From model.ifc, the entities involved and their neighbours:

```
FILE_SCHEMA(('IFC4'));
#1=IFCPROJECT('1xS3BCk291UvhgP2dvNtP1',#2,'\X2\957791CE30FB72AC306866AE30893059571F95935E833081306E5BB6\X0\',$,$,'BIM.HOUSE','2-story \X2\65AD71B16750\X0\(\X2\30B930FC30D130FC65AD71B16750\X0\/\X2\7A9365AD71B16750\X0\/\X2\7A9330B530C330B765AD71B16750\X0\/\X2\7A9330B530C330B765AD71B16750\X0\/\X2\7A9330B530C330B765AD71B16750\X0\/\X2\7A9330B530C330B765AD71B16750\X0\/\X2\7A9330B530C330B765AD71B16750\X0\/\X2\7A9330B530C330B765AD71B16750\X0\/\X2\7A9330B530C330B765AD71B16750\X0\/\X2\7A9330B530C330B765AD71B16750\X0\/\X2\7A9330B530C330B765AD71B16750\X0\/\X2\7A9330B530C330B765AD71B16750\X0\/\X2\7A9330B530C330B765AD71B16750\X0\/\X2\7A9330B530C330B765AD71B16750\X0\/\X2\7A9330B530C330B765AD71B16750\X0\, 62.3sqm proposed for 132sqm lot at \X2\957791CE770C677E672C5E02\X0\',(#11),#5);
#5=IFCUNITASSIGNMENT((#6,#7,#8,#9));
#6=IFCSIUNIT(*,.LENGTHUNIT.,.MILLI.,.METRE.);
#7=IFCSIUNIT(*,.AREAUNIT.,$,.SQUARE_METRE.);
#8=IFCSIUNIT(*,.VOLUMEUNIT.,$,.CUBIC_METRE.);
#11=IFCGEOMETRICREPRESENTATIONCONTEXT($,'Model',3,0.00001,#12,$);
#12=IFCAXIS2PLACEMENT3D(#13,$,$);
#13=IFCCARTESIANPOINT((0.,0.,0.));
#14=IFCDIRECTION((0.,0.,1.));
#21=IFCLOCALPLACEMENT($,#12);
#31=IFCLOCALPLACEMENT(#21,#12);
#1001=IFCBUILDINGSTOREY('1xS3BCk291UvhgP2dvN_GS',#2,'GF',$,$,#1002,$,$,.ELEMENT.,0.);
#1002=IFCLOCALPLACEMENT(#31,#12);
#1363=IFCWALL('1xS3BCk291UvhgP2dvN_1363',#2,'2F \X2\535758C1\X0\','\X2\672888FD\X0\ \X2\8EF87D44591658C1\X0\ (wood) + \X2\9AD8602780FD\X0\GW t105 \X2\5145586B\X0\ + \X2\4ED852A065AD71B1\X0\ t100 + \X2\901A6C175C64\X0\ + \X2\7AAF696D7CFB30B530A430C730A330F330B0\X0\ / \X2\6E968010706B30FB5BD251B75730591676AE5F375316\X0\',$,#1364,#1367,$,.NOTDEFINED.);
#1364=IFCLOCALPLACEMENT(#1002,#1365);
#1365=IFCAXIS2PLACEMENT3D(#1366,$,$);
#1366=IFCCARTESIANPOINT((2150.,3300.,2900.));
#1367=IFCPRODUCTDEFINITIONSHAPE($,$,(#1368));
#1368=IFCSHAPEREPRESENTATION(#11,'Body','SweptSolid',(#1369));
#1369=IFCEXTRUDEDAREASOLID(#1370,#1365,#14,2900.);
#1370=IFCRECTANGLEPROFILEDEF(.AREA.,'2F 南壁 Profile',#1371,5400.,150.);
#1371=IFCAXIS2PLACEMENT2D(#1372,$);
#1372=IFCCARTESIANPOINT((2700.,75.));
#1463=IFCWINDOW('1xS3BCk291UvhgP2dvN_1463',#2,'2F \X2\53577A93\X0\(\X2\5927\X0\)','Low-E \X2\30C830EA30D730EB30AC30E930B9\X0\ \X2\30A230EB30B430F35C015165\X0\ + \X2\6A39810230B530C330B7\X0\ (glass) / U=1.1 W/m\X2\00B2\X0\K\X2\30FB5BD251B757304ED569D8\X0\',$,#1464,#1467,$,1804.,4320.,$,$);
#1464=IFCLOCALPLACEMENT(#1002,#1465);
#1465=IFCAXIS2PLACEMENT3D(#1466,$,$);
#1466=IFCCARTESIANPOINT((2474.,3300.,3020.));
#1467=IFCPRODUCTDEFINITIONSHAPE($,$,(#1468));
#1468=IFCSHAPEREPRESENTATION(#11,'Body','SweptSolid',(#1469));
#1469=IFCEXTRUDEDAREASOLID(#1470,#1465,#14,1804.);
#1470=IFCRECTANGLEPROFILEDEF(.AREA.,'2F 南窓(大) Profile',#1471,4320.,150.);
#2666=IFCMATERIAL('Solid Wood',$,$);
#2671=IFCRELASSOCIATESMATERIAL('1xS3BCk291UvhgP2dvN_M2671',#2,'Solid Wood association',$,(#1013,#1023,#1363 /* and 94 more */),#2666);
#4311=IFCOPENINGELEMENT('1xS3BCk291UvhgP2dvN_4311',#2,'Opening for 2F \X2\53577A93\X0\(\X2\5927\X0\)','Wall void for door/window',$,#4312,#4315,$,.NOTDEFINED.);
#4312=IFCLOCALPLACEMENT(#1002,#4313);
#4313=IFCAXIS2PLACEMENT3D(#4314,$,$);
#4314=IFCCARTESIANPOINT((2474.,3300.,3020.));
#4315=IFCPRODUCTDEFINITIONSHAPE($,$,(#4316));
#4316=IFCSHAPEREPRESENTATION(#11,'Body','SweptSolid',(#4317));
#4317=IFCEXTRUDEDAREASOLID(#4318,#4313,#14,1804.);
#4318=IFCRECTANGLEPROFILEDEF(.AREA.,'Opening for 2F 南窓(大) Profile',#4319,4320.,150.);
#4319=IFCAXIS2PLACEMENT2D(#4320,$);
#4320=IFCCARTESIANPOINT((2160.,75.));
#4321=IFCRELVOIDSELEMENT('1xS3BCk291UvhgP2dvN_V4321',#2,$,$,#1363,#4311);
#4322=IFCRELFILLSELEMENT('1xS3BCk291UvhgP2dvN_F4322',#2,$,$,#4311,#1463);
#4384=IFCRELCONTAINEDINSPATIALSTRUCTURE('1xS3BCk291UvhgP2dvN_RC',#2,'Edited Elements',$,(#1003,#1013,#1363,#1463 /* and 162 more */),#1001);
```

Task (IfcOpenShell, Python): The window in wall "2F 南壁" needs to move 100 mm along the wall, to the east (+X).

```python
import ifcopenshell
import ifcopenshell.api.geometry
import ifcopenshell.util.placement

model = ifcopenshell.open("model.ifc")

window = model.by_guid("1xS3BCk291UvhgP2dvN_1463")
opening = window.FillsVoids[0].RelatingOpeningElement
wall = opening.VoidsElements[0].RelatingBuildingElement

wall_matrix = ifcopenshell.util.placement.get_local_placement(wall.ObjectPlacement)
shift = wall_matrix[:3, 0] * 100.0
before = ifcopenshell.util.placement.get_local_placement(window.ObjectPlacement)[:3, 3].copy()

# The window is not placed relative to its opening, so move both.
for product in (opening, window):
    matrix = ifcopenshell.util.placement.get_local_placement(product.ObjectPlacement)
    matrix[:3, 3] += shift
    ifcopenshell.api.geometry.edit_object_placement(model, product=product, matrix=matrix, is_si=False)

after = ifcopenshell.util.placement.get_local_placement(window.ObjectPlacement)[:3, 3]
print("window moved by", (after - before).round(3) + 0.0)

model.write("model_updated.ifc")
```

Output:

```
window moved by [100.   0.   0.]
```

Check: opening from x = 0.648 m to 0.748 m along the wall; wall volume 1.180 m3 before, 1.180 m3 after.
